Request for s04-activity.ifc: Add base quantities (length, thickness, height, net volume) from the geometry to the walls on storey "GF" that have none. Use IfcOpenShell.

First a look at what the model holds.

```python
import ifcopenshell
import ifcopenshell.util.element
import ifcopenshell.util.unit

model = ifcopenshell.open("s04-activity.ifc")
print(model.schema)
for unit_type in ("LENGTHUNIT", "AREAUNIT", "VOLUMEUNIT"):
    print(unit_type, ifcopenshell.util.unit.calculate_unit_scale(model, unit_type))
storey = next(s for s in model.by_type("IfcBuildingStorey") if s.Name == "GF")
walls = [e for e in ifcopenshell.util.element.get_decomposition(storey) if e.is_a("IfcWall")]
for e in sorted(walls, key=lambda e: e.id()):
    print(e.id(), e.is_a(), e.Name, list(ifcopenshell.util.element.get_psets(e, qtos_only=True)), sep=" | ")
```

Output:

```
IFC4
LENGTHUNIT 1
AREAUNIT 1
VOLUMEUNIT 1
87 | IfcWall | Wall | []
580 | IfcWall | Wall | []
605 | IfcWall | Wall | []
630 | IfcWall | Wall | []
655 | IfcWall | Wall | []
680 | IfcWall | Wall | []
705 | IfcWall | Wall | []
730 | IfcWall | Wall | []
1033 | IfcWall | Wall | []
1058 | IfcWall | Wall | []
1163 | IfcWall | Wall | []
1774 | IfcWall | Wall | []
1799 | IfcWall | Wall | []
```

```python
import ifcopenshell
import ifcopenshell.api.pset
import ifcopenshell.geom
import ifcopenshell.util.element
import ifcopenshell.util.shape
import ifcopenshell.util.unit

model = ifcopenshell.open("s04-activity.ifc")
unit_scale = ifcopenshell.util.unit.calculate_unit_scale(model)
volume_scale = ifcopenshell.util.unit.calculate_unit_scale(model, "VOLUMEUNIT")
settings = ifcopenshell.geom.settings()

storey = next(s for s in model.by_type("IfcBuildingStorey") if s.Name == "GF")
walls = [e for e in ifcopenshell.util.element.get_decomposition(storey) if e.is_a("IfcWall")]

for e in sorted(walls, key=lambda e: e.id()):
    if ifcopenshell.util.element.get_psets(e, qtos_only=True, should_inherit=False):
        continue
    # Geometry comes back in metres, in the element's own axes.
    shape = ifcopenshell.geom.create_shape(settings, e)
    values = {
        "Length": ifcopenshell.util.shape.get_x(shape.geometry) / unit_scale,
        "Width": ifcopenshell.util.shape.get_y(shape.geometry) / unit_scale,
        "Height": ifcopenshell.util.shape.get_z(shape.geometry) / unit_scale,
        "NetVolume": ifcopenshell.util.shape.get_volume(shape.geometry) / volume_scale,
    }
    qto = ifcopenshell.api.pset.add_qto(model, product=e, name="Qto_WallBaseQuantities")
    ifcopenshell.api.pset.edit_qto(model, qto=qto, properties=values)
    print(e.id(), {k: round(v, 3) for k, v in values.items()})

model.write("s04-activity_rev.ifc")
```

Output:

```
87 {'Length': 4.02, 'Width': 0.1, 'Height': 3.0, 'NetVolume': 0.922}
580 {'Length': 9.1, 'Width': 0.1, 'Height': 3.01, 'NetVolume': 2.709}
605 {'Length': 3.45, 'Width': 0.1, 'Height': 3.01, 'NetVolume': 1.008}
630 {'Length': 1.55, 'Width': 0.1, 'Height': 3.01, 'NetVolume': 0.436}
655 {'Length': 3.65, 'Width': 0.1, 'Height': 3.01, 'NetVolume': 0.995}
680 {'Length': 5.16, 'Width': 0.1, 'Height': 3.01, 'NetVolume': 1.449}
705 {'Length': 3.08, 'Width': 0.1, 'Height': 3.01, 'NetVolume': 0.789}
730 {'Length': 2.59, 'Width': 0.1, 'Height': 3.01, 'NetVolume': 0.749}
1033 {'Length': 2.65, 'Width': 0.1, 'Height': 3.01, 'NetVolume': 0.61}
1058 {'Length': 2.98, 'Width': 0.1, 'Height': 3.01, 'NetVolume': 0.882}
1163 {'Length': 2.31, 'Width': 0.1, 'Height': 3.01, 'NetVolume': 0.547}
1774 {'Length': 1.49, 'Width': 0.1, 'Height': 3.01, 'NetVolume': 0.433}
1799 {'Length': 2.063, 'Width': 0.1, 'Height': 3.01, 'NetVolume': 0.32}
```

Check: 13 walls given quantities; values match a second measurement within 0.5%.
